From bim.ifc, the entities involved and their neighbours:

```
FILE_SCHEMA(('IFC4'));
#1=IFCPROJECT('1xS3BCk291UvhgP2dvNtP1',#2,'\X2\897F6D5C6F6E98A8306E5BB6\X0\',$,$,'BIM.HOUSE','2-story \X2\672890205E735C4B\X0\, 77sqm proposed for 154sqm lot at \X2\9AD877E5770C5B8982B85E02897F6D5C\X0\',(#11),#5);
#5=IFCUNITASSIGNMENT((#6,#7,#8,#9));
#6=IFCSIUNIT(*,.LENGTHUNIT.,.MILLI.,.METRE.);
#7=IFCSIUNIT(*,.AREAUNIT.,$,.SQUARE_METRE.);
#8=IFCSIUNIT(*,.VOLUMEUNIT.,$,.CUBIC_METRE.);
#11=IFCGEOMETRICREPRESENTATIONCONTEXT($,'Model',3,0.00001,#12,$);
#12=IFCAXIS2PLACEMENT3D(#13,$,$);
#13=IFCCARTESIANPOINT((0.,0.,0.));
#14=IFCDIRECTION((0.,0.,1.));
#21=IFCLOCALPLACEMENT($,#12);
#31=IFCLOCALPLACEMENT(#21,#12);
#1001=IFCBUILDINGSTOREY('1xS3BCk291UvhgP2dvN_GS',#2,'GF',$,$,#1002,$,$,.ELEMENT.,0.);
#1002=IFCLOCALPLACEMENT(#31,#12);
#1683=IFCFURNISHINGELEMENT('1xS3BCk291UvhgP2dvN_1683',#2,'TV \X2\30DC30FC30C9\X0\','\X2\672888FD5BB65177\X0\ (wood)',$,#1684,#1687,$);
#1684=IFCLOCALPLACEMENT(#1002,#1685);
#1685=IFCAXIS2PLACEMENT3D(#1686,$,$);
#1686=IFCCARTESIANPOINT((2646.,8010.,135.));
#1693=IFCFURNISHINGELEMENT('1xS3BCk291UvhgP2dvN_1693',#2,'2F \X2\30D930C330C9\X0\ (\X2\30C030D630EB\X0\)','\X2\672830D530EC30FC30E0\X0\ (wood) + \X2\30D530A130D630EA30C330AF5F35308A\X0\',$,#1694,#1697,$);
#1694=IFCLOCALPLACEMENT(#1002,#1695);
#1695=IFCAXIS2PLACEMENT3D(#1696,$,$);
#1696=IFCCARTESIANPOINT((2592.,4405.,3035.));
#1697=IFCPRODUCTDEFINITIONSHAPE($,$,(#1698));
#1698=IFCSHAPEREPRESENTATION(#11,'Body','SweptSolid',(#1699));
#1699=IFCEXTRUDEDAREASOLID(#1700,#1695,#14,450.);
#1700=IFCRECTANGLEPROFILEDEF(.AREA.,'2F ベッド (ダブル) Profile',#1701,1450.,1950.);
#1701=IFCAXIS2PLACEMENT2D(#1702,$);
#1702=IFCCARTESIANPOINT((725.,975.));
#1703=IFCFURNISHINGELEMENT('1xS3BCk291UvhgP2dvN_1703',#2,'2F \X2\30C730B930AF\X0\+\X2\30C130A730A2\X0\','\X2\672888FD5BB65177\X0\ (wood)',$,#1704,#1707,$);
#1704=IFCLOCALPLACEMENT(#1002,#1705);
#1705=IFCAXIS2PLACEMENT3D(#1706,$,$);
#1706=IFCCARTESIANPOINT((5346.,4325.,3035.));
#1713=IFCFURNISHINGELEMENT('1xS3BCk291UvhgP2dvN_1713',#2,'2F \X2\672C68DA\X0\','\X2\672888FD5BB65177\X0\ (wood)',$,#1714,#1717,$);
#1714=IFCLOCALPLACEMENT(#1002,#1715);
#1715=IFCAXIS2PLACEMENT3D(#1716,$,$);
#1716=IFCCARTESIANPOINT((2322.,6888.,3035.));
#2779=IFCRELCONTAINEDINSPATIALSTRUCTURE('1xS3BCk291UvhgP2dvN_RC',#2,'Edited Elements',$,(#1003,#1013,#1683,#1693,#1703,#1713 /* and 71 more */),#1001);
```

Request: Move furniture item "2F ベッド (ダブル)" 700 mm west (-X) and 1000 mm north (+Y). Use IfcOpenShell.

```python
import ifcopenshell
import ifcopenshell.api.geometry
import ifcopenshell.util.placement

model = ifcopenshell.open("bim.ifc")

item = model.by_id(1693)
matrix = ifcopenshell.util.placement.get_local_placement(item.ObjectPlacement)
matrix[0, 3] -= 700.0
matrix[1, 3] += 1000.0
ifcopenshell.api.geometry.edit_object_placement(model, product=item, matrix=matrix, is_si=False)

print(ifcopenshell.util.placement.get_local_placement(item.ObjectPlacement).round(3) + 0.0)

model.write("bim_edited.ifc")
```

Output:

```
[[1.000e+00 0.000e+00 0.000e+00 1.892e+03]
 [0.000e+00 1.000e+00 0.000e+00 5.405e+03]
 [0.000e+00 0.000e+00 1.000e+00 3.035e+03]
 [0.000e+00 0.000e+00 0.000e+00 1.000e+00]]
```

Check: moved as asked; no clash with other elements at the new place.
